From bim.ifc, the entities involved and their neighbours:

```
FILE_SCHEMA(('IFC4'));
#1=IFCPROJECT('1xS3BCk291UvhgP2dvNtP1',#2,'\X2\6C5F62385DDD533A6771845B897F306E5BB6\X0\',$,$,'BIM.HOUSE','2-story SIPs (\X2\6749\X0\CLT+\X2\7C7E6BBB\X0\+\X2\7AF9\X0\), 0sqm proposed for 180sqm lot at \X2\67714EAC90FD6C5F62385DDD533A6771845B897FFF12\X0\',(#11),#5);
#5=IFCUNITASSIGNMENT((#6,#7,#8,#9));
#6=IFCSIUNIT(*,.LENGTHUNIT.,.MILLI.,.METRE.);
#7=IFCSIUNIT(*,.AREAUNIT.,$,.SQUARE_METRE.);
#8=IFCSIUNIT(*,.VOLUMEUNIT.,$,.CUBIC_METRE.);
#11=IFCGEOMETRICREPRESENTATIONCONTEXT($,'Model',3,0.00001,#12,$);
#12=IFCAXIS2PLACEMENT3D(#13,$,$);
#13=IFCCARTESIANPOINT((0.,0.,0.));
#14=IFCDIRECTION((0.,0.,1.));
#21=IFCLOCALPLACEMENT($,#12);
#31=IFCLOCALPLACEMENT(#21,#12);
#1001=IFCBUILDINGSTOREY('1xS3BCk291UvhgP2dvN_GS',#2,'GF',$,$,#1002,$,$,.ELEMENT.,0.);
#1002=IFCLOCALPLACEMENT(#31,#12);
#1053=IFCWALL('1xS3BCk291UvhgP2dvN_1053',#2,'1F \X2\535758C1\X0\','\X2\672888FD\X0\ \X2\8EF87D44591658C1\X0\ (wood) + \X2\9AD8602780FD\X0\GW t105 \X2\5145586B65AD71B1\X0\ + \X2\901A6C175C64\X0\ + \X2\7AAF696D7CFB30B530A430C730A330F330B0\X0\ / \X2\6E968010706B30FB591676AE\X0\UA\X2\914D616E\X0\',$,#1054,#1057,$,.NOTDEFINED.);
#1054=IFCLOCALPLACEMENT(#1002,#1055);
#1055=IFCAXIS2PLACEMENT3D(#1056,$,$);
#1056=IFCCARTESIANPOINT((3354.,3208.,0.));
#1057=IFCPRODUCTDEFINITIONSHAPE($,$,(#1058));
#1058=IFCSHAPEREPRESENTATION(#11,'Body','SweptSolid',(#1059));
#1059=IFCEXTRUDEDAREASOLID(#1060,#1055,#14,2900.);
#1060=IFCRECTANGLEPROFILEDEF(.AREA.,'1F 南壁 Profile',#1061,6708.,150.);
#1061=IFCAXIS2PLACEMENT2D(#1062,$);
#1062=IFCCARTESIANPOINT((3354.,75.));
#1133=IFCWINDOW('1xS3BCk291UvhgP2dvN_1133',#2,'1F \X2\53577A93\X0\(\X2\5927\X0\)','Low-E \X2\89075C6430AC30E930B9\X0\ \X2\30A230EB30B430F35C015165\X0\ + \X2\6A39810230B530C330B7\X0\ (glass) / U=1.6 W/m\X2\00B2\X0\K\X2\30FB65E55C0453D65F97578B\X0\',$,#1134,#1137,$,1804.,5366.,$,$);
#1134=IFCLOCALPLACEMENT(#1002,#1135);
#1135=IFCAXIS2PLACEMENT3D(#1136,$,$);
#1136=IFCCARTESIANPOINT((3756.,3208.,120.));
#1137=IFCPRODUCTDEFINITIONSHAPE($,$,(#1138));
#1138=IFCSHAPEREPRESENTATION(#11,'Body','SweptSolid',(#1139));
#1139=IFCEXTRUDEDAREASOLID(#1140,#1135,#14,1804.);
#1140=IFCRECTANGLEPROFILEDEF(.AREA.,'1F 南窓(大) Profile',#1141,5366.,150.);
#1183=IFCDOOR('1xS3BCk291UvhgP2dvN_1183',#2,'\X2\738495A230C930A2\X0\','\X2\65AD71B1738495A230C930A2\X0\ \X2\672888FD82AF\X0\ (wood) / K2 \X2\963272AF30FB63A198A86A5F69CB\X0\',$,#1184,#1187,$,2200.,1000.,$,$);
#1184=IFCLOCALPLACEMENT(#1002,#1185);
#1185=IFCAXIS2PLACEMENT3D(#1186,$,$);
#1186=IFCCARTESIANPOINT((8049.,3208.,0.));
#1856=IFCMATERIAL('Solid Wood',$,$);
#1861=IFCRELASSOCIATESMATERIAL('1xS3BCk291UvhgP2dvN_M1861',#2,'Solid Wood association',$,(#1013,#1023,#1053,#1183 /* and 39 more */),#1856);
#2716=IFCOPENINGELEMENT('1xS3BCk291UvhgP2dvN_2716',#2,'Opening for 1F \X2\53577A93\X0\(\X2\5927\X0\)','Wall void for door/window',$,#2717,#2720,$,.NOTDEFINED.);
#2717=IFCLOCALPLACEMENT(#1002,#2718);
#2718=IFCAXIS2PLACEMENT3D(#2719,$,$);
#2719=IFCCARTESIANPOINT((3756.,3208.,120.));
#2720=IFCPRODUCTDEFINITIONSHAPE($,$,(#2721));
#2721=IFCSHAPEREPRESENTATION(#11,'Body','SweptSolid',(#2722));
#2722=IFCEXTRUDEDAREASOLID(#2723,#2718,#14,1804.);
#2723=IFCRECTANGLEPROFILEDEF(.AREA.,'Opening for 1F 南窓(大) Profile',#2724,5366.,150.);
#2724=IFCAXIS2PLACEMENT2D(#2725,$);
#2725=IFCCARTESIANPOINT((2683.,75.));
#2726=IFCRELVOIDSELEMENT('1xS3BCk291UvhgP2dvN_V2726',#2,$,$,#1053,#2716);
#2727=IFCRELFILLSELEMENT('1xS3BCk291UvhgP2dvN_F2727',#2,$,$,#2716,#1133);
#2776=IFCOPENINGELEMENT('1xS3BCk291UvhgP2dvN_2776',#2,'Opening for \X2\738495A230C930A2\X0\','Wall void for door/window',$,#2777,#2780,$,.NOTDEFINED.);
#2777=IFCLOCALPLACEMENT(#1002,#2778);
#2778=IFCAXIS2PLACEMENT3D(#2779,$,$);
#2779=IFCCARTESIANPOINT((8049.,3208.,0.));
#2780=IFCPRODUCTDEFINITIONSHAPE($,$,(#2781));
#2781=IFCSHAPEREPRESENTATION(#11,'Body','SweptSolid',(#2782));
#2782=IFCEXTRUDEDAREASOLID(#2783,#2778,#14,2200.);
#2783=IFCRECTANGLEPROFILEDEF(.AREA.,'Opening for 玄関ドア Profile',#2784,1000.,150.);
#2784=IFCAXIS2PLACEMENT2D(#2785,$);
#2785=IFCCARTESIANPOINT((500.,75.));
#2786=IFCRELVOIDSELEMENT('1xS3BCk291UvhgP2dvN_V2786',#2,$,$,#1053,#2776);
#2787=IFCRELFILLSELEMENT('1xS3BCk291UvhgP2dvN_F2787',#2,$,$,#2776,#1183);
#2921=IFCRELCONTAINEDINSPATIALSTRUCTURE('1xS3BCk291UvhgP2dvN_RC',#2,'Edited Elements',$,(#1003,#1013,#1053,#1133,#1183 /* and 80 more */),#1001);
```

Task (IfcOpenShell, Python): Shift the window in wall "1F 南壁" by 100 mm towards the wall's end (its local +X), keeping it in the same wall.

```python
import ifcopenshell
import ifcopenshell.api.geometry
import ifcopenshell.util.placement
import ifcopenshell.util.unit

model = ifcopenshell.open("bim.ifc")
unit_scale = ifcopenshell.util.unit.calculate_unit_scale(model)

window = model.by_id(1133)
opening = window.FillsVoids[0].RelatingOpeningElement
wall = opening.VoidsElements[0].RelatingBuildingElement

wall_matrix = ifcopenshell.util.placement.get_local_placement(wall.ObjectPlacement)
shift = wall_matrix[:3, 0] * 0.1 / unit_scale
before = ifcopenshell.util.placement.get_local_placement(window.ObjectPlacement)[:3, 3].copy()

# The window is not placed relative to its opening, so move both.
for product in (opening, window):
    matrix = ifcopenshell.util.placement.get_local_placement(product.ObjectPlacement)
    matrix[:3, 3] += shift
    ifcopenshell.api.geometry.edit_object_placement(model, product=product, matrix=matrix, is_si=False)

after = ifcopenshell.util.placement.get_local_placement(window.ObjectPlacement)[:3, 3]
print("window moved by", (after - before).round(3) + 0.0)

model.write("bim_updated.ifc")
```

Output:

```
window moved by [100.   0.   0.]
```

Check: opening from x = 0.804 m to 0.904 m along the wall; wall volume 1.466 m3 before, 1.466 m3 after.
